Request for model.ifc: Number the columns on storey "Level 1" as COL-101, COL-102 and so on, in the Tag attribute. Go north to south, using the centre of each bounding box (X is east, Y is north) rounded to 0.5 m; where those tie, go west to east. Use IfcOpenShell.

First a look at what the model holds.

```python
import ifcopenshell
import ifcopenshell.util.element
import ifcopenshell.util.placement

model = ifcopenshell.open("model.ifc")
print(model.schema)
storey = next(s for s in model.by_type("IfcBuildingStorey") if s.Name == "Level 1")
columns = [e for e in ifcopenshell.util.element.get_decomposition(storey) if e.is_a("IfcColumn")]
for e in sorted(columns, key=lambda e: e.id()):
    origin = ifcopenshell.util.placement.get_local_placement(e.ObjectPlacement)[:3, 3]
    print(e.id(), e.Tag, e.Name, origin.round(2) + 0.0, sep=" | ")
```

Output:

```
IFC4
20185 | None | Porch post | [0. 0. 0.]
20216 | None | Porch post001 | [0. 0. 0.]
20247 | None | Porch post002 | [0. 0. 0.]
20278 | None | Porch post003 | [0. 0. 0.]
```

```python
import ifcopenshell
import ifcopenshell.geom
import ifcopenshell.util.element
import ifcopenshell.util.shape

model = ifcopenshell.open("model.ifc")
settings = ifcopenshell.geom.settings()
settings.set("use-world-coords", True)


def centre(element):
    shape = ifcopenshell.geom.create_shape(settings, element)
    return ifcopenshell.util.shape.get_bbox_centroid(shape.geometry)


storey = next(s for s in model.by_type("IfcBuildingStorey") if s.Name == "Level 1")
columns = [e for e in ifcopenshell.util.element.get_decomposition(storey) if e.is_a("IfcColumn")]

# Insertion points can sit at a corner or the storey origin, so sort by the geometry (in metres).
centres = {e: centre(e) for e in columns}
columns.sort(key=lambda e: (-round(centres[e][1] / 0.5), centres[e][0]))

for i, e in enumerate(columns, start=1):
    number = f"COL-1{i:02d}"
    e.Tag = number
    print(e.id(), number)

model.write("model_v2.ifc")
```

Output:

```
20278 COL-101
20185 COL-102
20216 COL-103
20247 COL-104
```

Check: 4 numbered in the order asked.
